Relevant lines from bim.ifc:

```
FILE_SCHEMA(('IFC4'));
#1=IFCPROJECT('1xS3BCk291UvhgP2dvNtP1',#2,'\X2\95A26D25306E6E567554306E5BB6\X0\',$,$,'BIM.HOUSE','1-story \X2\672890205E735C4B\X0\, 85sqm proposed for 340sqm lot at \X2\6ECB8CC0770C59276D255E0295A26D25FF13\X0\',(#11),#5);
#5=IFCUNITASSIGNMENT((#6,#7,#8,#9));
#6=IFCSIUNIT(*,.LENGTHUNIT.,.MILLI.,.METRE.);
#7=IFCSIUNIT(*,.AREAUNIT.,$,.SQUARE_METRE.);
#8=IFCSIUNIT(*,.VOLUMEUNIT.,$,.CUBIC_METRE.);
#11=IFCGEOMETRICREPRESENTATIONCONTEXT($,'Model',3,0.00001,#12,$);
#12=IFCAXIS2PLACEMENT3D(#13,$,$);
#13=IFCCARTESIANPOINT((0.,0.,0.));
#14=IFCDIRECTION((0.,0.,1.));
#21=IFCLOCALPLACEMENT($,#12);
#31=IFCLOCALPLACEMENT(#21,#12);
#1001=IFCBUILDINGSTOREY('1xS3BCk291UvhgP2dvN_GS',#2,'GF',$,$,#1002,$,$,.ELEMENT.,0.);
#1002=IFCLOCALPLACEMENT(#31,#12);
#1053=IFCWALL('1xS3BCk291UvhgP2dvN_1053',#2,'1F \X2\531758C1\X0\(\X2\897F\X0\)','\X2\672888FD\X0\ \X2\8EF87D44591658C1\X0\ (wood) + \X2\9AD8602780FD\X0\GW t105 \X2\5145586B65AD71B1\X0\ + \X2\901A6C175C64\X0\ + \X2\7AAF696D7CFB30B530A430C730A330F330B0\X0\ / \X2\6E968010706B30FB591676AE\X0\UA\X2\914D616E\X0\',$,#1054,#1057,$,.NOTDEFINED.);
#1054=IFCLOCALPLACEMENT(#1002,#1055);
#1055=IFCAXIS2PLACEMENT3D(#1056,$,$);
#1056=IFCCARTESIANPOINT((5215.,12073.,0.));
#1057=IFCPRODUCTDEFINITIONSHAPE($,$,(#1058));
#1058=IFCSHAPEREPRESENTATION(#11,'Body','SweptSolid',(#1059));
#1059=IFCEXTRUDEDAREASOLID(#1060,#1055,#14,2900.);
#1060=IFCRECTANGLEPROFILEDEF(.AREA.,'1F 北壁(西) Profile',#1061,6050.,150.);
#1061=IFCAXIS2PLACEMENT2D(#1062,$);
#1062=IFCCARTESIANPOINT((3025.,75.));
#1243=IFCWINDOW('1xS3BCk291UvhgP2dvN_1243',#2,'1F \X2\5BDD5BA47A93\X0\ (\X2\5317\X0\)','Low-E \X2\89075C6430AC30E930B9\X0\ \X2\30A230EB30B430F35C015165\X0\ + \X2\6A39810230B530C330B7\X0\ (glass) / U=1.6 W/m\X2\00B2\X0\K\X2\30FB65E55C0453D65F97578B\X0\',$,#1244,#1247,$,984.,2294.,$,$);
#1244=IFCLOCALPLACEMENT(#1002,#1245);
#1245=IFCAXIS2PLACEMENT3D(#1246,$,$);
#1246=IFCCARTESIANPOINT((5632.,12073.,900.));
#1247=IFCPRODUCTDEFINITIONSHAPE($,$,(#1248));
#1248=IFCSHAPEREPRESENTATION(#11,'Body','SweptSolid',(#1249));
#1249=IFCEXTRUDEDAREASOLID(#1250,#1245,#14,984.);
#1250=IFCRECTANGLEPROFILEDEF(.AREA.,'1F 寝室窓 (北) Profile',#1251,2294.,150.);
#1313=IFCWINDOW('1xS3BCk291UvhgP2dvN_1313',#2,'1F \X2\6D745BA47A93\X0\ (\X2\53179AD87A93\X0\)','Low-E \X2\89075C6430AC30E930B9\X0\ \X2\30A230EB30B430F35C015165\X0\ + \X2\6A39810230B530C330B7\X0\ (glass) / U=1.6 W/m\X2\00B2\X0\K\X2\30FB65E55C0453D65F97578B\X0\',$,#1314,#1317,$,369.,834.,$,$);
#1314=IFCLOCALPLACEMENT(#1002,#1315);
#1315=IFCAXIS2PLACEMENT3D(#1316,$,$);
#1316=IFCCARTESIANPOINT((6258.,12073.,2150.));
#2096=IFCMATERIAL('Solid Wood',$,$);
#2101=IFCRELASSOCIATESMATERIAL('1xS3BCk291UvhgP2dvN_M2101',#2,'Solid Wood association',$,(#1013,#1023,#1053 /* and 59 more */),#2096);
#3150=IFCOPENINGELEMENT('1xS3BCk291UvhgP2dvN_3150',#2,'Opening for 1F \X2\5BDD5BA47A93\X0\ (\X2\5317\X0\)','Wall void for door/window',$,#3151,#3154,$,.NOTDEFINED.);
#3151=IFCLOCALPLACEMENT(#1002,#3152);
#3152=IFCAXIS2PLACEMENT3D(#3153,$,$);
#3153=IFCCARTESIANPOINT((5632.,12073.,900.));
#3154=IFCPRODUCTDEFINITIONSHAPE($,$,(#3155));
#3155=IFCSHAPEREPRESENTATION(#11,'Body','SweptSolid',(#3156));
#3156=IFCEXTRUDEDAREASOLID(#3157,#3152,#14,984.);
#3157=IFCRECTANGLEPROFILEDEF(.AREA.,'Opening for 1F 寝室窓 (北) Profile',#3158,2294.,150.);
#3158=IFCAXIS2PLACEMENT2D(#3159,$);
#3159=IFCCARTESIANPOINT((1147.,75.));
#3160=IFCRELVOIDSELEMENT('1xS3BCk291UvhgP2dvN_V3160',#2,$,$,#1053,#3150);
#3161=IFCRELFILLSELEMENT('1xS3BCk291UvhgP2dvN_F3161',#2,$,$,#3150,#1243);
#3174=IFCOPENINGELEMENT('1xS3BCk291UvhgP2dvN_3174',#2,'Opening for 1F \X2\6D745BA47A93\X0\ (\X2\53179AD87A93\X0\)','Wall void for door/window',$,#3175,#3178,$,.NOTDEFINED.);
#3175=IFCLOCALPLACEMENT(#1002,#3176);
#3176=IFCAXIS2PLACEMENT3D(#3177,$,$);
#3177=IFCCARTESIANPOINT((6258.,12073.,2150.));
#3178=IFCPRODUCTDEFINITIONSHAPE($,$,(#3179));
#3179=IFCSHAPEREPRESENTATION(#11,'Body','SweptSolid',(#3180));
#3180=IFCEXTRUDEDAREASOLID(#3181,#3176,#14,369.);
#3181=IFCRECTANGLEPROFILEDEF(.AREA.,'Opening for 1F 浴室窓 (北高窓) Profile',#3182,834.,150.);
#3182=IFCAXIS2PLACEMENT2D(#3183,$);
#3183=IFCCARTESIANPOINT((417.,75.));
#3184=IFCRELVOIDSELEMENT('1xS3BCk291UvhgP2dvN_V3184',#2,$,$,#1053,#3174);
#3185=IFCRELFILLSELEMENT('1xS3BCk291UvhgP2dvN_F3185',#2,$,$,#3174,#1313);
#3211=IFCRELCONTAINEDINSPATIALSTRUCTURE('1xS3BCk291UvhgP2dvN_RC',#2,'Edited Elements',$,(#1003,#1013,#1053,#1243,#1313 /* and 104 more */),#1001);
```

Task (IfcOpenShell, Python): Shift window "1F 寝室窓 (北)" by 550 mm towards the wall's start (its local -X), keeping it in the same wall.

```python
import ifcopenshell
import ifcopenshell.api.geometry
import ifcopenshell.util.placement
import ifcopenshell.util.unit

model = ifcopenshell.open("bim.ifc")
unit_scale = ifcopenshell.util.unit.calculate_unit_scale(model)

window = model.by_id(1243)
opening = window.FillsVoids[0].RelatingOpeningElement
wall = opening.VoidsElements[0].RelatingBuildingElement

wall_matrix = ifcopenshell.util.placement.get_local_placement(wall.ObjectPlacement)
shift = wall_matrix[:3, 0] * -0.55 / unit_scale
before = ifcopenshell.util.placement.get_local_placement(window.ObjectPlacement)[:3, 3].copy()

# The window is not placed relative to its opening, so move both.
for product in (opening, window):
    matrix = ifcopenshell.util.placement.get_local_placement(product.ObjectPlacement)
    matrix[:3, 3] += shift
    ifcopenshell.api.geometry.edit_object_placement(model, product=product, matrix=matrix, is_si=False)

after = ifcopenshell.util.placement.get_local_placement(window.ObjectPlacement)[:3, 3]
print("window moved by", (after - before).round(3) + 0.0)

model.write("bim_edited.ifc")
```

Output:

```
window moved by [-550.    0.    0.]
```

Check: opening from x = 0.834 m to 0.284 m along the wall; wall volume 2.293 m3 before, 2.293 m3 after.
